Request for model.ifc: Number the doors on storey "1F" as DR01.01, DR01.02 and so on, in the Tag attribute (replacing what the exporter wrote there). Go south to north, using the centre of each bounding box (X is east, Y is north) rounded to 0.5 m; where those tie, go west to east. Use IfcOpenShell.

First a look at what the model holds.

```python
import ifcopenshell
import ifcopenshell.util.element
import ifcopenshell.util.placement

model = ifcopenshell.open("model.ifc")
print(model.schema)
storey = next(s for s in model.by_type("IfcBuildingStorey") if s.Name == "1F")
doors = [e for e in ifcopenshell.util.element.get_decomposition(storey) if e.is_a("IfcDoor")]
for e in sorted(doors, key=lambda e: e.id()):
    origin = ifcopenshell.util.placement.get_local_placement(e.ObjectPlacement)[:3, 3]
    print(e.id(), e.Tag, e.Name, origin.round(2) + 0.0, sep=" | ")
```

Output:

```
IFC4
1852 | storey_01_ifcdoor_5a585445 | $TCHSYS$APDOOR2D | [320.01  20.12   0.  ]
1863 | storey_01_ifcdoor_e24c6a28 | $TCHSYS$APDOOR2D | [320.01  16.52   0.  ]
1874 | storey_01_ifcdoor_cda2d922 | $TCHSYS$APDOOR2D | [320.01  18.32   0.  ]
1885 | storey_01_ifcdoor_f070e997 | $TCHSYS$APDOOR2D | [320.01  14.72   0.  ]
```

```python
import ifcopenshell
import ifcopenshell.geom
import ifcopenshell.util.element
import ifcopenshell.util.shape

model = ifcopenshell.open("model.ifc")
settings = ifcopenshell.geom.settings()
settings.set("use-world-coords", True)


def centre(element):
    shape = ifcopenshell.geom.create_shape(settings, element)
    return ifcopenshell.util.shape.get_bbox_centroid(shape.geometry)


storey = next(s for s in model.by_type("IfcBuildingStorey") if s.Name == "1F")
doors = [e for e in ifcopenshell.util.element.get_decomposition(storey) if e.is_a("IfcDoor")]

# Insertion points can sit at a corner or the storey origin, so sort by the geometry (in metres).
centres = {e: centre(e) for e in doors}
doors.sort(key=lambda e: (round(centres[e][1] / 0.5), centres[e][0]))

for i, e in enumerate(doors, start=1):
    number = f"DR01.{i:02d}"
    e.Tag = number
    print(e.id(), number)

model.write("model_v2.ifc")
```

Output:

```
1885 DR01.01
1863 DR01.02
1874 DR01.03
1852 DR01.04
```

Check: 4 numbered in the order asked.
